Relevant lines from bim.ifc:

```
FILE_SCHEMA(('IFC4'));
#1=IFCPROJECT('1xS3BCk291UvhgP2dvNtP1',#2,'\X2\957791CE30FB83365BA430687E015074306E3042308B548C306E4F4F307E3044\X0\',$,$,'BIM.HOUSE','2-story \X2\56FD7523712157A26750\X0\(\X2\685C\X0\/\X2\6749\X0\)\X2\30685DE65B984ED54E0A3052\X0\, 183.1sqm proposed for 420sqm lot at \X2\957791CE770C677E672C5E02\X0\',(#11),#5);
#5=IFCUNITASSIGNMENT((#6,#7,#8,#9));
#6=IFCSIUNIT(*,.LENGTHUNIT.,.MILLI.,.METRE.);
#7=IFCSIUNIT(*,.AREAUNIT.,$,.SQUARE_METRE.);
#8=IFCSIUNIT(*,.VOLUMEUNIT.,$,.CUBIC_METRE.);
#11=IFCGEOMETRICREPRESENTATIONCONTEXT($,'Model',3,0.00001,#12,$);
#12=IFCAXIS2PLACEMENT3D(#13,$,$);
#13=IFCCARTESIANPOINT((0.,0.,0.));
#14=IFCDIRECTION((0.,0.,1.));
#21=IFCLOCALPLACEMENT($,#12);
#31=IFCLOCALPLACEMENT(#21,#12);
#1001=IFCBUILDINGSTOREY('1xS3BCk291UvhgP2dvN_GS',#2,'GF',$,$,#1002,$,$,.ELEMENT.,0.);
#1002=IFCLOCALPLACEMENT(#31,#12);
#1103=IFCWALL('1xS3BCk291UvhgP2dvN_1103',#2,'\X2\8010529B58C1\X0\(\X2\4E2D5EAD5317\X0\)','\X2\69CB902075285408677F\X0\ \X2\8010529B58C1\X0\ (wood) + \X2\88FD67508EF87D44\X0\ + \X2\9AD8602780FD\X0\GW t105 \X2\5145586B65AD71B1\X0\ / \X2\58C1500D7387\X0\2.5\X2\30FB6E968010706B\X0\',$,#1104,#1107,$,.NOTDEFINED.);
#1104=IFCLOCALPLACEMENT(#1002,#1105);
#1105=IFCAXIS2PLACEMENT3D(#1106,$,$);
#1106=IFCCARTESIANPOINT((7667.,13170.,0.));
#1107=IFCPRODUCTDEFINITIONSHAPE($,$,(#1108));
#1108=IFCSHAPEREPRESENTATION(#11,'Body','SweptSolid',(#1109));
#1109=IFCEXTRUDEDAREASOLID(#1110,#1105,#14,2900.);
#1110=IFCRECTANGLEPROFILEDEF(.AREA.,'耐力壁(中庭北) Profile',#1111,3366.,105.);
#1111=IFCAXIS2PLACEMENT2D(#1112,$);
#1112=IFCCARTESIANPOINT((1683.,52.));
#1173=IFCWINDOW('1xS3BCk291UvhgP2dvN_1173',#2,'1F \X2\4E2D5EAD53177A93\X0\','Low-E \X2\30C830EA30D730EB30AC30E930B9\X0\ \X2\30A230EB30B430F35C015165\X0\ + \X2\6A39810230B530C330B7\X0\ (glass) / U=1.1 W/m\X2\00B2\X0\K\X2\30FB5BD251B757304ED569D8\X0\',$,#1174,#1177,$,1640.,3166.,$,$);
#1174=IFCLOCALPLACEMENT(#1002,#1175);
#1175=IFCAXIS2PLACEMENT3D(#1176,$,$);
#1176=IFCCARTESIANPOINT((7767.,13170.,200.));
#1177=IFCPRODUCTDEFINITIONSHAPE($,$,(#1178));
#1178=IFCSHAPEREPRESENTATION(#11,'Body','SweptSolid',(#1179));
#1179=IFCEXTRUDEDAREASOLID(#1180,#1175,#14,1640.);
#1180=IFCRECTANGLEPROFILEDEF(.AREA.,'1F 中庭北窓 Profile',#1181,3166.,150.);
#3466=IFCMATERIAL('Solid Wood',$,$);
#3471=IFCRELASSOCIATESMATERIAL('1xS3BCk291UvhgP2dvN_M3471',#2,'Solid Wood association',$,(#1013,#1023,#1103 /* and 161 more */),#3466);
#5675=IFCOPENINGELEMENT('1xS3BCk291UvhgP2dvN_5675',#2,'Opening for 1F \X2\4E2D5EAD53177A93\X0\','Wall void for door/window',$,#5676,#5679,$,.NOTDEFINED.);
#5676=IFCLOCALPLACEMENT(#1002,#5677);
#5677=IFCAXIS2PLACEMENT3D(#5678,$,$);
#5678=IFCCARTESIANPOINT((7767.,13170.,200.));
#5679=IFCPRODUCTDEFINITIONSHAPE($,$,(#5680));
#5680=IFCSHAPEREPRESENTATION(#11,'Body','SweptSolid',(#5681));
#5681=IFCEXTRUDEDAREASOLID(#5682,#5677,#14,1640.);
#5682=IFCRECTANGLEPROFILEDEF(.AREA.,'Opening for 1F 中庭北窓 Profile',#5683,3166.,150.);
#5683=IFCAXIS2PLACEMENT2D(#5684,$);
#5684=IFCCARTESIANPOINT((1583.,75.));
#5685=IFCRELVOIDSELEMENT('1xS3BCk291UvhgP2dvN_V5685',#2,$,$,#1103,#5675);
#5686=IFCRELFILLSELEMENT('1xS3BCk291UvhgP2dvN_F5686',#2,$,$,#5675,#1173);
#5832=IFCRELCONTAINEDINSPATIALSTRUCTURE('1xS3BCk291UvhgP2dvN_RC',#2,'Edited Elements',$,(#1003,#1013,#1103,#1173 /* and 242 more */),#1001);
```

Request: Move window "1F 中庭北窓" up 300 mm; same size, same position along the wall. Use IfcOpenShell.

```python
import numpy as np
import ifcopenshell
import ifcopenshell.api.geometry
import ifcopenshell.util.placement
import ifcopenshell.util.unit

model = ifcopenshell.open("bim.ifc")
unit_scale = ifcopenshell.util.unit.calculate_unit_scale(model)

window = model.by_guid("1xS3BCk291UvhgP2dvN_1173")
opening = window.FillsVoids[0].RelatingOpeningElement
dz = 300.0

shift = np.array([0.0, 0.0, dz])
# The window is not placed relative to its opening, so move both.
for product in (opening, window):
    matrix = ifcopenshell.util.placement.get_local_placement(product.ObjectPlacement)
    matrix[:3, 3] += shift
    ifcopenshell.api.geometry.edit_object_placement(model, product=product, matrix=matrix, is_si=False)

print(f"moved by {dz * unit_scale:+.3f} m")

model.write("bim_v2.ifc")
```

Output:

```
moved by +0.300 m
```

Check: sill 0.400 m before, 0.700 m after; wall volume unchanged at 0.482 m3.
